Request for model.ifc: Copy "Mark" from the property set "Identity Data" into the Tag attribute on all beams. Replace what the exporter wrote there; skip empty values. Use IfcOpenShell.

First a look at what the model holds.

```python
import ifcopenshell
import ifcopenshell.util.element

model = ifcopenshell.open("model.ifc")
print(model.schema)
beams = model.by_type("IfcBeam")
print(len(beams), "beams")
for e in beams[:8]:
    source = ifcopenshell.util.element.get_pset(e, "Identity Data", "Mark")
    target = e.Tag
    print(e.id(), repr(source), repr(target), sep=" | ")
```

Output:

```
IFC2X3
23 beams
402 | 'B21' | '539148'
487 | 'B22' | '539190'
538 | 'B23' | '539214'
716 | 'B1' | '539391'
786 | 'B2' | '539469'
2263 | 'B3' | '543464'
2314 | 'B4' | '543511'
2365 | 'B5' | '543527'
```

```python
import ifcopenshell
import ifcopenshell.util.element

model = ifcopenshell.open("model.ifc")

count = 0
for e in model.by_type("IfcBeam"):
    value = ifcopenshell.util.element.get_pset(e, "Identity Data", "Mark")
    current = e.Tag
    if not value or not value.strip() or current == value:
        continue
    e.Tag = value
    count += 1

print(count, "beams updated")

model.write("model_updated.ifc")
```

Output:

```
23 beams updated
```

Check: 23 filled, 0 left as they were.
